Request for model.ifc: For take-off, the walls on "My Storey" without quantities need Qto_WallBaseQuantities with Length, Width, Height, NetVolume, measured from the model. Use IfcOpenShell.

First a look at what the model holds.

```python
import ifcopenshell
import ifcopenshell.util.element
import ifcopenshell.util.unit

model = ifcopenshell.open("model.ifc")
print(model.schema)
for unit_type in ("LENGTHUNIT", "AREAUNIT", "VOLUMEUNIT"):
    print(unit_type, ifcopenshell.util.unit.calculate_unit_scale(model, unit_type))
storey = next(s for s in model.by_type("IfcBuildingStorey") if s.Name == "My Storey")
walls = [e for e in ifcopenshell.util.element.get_decomposition(storey) if e.is_a("IfcWall")]
for e in sorted(walls, key=lambda e: e.id()):
    print(e.id(), e.is_a(), e.Name, list(ifcopenshell.util.element.get_psets(e, qtos_only=True)), sep=" | ")
```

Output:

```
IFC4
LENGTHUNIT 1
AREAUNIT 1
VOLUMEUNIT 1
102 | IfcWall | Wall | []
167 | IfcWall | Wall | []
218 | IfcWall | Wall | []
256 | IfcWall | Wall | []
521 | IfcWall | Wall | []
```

```python
import ifcopenshell
import ifcopenshell.api.pset
import ifcopenshell.geom
import ifcopenshell.util.element
import ifcopenshell.util.shape
import ifcopenshell.util.unit

model = ifcopenshell.open("model.ifc")
unit_scale = ifcopenshell.util.unit.calculate_unit_scale(model)
volume_scale = ifcopenshell.util.unit.calculate_unit_scale(model, "VOLUMEUNIT")
settings = ifcopenshell.geom.settings()

storey = next(s for s in model.by_type("IfcBuildingStorey") if s.Name == "My Storey")
walls = [e for e in ifcopenshell.util.element.get_decomposition(storey) if e.is_a("IfcWall")]

for e in sorted(walls, key=lambda e: e.id()):
    if ifcopenshell.util.element.get_psets(e, qtos_only=True, should_inherit=False):
        continue
    # Geometry comes back in metres, in the element's own axes.
    shape = ifcopenshell.geom.create_shape(settings, e)
    values = {
        "Length": ifcopenshell.util.shape.get_x(shape.geometry) / unit_scale,
        "Width": ifcopenshell.util.shape.get_y(shape.geometry) / unit_scale,
        "Height": ifcopenshell.util.shape.get_z(shape.geometry) / unit_scale,
        "NetVolume": ifcopenshell.util.shape.get_volume(shape.geometry) / volume_scale,
    }
    qto = ifcopenshell.api.pset.add_qto(model, product=e, name="Qto_WallBaseQuantities")
    ifcopenshell.api.pset.edit_qto(model, qto=qto, properties=values)
    print(e.id(), {k: round(v, 3) for k, v in values.items()})

model.write("model-out.ifc")
```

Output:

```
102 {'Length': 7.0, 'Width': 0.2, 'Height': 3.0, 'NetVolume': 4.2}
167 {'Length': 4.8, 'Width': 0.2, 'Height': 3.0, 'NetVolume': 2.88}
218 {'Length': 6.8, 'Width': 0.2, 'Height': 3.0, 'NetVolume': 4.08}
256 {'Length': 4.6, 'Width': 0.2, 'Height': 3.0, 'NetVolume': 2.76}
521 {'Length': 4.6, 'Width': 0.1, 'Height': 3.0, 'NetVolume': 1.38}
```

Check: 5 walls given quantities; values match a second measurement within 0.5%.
